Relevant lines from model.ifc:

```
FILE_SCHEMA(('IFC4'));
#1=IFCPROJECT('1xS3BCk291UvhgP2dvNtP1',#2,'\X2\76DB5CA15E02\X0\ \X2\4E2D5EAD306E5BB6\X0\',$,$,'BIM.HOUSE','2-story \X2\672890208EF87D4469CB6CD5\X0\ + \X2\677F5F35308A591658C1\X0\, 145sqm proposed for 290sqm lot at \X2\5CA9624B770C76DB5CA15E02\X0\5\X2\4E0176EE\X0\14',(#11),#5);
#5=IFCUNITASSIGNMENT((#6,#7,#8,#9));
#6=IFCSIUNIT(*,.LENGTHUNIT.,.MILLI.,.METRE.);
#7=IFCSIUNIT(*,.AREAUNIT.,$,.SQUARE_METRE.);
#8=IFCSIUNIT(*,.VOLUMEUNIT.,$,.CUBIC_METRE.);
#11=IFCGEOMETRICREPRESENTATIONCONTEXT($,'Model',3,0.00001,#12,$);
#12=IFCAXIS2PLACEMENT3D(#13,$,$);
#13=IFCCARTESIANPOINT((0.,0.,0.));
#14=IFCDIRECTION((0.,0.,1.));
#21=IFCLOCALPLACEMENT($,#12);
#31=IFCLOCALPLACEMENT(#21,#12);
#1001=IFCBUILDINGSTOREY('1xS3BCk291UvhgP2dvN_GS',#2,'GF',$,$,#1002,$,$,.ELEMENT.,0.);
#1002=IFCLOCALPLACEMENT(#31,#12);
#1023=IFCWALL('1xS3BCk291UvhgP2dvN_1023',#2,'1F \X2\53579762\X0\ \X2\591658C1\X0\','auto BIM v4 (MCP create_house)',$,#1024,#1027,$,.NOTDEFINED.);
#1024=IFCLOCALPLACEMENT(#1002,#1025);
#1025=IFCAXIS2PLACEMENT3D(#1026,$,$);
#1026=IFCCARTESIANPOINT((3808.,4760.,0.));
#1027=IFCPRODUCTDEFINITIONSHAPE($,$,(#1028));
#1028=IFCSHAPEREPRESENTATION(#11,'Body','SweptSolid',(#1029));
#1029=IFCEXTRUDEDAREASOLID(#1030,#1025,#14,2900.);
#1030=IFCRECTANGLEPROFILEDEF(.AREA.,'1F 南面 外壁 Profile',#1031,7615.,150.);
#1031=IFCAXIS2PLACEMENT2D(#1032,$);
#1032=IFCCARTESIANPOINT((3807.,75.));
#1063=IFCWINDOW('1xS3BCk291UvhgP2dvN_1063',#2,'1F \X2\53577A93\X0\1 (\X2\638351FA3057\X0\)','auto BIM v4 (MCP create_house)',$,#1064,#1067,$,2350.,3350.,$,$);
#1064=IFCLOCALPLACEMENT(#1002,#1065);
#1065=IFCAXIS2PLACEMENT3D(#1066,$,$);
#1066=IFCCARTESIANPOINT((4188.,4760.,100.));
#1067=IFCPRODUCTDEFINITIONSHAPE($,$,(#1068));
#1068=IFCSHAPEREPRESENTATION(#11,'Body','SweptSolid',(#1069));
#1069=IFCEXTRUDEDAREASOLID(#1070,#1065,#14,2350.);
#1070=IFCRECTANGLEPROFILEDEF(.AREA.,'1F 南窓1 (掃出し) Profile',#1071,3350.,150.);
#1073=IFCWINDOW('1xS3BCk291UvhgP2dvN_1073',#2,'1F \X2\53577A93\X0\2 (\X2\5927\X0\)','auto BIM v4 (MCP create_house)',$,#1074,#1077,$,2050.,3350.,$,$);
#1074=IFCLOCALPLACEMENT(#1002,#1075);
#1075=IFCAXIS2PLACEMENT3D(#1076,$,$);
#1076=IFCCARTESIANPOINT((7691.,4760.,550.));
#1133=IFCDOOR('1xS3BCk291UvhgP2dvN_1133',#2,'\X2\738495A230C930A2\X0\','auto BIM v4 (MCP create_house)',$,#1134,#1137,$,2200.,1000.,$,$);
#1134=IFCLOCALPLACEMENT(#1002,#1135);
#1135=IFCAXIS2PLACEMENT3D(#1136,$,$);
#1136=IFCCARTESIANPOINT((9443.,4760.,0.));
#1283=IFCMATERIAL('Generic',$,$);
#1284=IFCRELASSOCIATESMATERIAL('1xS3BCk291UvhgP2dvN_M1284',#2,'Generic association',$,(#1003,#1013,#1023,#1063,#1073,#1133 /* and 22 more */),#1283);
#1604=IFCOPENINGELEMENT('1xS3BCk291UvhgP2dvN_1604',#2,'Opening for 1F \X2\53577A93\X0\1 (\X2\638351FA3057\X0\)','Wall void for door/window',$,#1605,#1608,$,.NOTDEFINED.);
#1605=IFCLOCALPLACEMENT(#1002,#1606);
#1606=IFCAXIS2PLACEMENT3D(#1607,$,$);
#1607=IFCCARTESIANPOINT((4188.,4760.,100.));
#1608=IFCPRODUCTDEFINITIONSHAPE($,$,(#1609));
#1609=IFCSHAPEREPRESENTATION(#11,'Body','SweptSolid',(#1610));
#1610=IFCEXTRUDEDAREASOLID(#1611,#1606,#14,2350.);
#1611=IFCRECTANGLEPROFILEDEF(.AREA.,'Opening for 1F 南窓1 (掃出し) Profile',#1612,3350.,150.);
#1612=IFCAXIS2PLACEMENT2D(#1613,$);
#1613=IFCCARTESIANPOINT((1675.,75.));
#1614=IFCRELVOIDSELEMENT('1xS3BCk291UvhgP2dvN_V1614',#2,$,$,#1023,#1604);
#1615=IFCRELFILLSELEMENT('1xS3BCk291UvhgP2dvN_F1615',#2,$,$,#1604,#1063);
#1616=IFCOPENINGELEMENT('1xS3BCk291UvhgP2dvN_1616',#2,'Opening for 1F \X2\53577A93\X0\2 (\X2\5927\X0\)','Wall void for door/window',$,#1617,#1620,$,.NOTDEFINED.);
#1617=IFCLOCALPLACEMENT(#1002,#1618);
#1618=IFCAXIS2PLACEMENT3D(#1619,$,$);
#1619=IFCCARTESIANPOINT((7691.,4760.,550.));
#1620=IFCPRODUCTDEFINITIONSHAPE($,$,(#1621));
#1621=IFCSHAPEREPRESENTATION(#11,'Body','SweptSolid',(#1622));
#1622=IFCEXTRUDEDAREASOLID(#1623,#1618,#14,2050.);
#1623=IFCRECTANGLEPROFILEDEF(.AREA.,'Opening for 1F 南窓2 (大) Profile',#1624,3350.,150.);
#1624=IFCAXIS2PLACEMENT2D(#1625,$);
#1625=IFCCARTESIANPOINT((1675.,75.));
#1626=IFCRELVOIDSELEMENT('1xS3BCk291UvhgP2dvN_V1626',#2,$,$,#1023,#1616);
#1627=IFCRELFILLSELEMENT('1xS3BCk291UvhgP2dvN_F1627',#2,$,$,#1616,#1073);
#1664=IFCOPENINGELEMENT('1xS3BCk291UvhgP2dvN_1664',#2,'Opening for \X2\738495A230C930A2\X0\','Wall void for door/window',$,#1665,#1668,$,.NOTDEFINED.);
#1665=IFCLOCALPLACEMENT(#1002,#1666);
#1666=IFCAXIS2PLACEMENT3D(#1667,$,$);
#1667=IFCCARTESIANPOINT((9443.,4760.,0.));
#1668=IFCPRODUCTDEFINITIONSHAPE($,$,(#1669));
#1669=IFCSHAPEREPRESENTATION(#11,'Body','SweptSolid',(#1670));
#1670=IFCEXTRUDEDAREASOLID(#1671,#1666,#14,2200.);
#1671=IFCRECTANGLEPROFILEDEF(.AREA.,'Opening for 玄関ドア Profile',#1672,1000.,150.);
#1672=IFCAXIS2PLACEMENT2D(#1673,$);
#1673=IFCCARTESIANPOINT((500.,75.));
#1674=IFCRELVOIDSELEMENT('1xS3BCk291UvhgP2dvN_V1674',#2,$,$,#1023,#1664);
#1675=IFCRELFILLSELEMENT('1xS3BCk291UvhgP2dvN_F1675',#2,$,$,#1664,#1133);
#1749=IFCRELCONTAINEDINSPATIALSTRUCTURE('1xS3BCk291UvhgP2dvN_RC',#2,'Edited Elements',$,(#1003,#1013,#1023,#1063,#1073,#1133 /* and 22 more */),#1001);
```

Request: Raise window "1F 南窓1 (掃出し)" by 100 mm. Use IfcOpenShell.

```python
import numpy as np
import ifcopenshell
import ifcopenshell.api.geometry
import ifcopenshell.util.placement
import ifcopenshell.util.unit

model = ifcopenshell.open("model.ifc")
unit_scale = ifcopenshell.util.unit.calculate_unit_scale(model)

window = model.by_guid("1xS3BCk291UvhgP2dvN_1063")
opening = window.FillsVoids[0].RelatingOpeningElement
dz = 100.0

shift = np.array([0.0, 0.0, dz])
# The window is not placed relative to its opening, so move both.
for product in (opening, window):
    matrix = ifcopenshell.util.placement.get_local_placement(product.ObjectPlacement)
    matrix[:3, 3] += shift
    ifcopenshell.api.geometry.edit_object_placement(model, product=product, matrix=matrix, is_si=False)

print(f"moved by {dz * unit_scale:+.3f} m")

model.write("model_updated.ifc")
```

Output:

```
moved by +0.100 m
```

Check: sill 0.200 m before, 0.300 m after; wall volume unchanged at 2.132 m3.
